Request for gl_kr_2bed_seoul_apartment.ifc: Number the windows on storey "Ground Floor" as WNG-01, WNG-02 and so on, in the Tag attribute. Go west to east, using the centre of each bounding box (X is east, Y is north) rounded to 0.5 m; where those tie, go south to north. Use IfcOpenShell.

First a look at what the model holds.

```python
import ifcopenshell
import ifcopenshell.util.element
import ifcopenshell.util.placement

model = ifcopenshell.open("gl_kr_2bed_seoul_apartment.ifc")
print(model.schema)
storey = next(s for s in model.by_type("IfcBuildingStorey") if s.Name == "Ground Floor")
windows = [e for e in ifcopenshell.util.element.get_decomposition(storey) if e.is_a("IfcWindow")]
for e in sorted(windows, key=lambda e: e.id()):
    origin = ifcopenshell.util.placement.get_local_placement(e.ObjectPlacement)[:3, 3]
    print(e.id(), e.Tag, e.Name, origin.round(2) + 0.0, sep=" | ")
```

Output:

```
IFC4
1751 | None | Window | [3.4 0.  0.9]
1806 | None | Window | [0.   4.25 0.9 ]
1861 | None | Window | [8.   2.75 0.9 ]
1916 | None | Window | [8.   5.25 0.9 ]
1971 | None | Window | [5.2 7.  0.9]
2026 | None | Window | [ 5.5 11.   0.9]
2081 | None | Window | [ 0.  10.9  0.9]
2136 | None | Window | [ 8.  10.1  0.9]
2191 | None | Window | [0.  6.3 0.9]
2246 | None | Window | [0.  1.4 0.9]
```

```python
import ifcopenshell
import ifcopenshell.geom
import ifcopenshell.util.element
import ifcopenshell.util.shape

model = ifcopenshell.open("gl_kr_2bed_seoul_apartment.ifc")
settings = ifcopenshell.geom.settings()
settings.set("use-world-coords", True)


def centre(element):
    shape = ifcopenshell.geom.create_shape(settings, element)
    return ifcopenshell.util.shape.get_bbox_centroid(shape.geometry)


storey = next(s for s in model.by_type("IfcBuildingStorey") if s.Name == "Ground Floor")
windows = [e for e in ifcopenshell.util.element.get_decomposition(storey) if e.is_a("IfcWindow")]

# Insertion points can sit at a corner or the storey origin, so sort by the geometry (in metres).
centres = {e: centre(e) for e in windows}
windows.sort(key=lambda e: (round(centres[e][0] / 0.5), centres[e][1]))

for i, e in enumerate(windows, start=1):
    number = f"WNG-{i:02d}"
    e.Tag = number
    print(e.id(), number)

model.write("gl_kr_2bed_seoul_apartment_updated.ifc")
```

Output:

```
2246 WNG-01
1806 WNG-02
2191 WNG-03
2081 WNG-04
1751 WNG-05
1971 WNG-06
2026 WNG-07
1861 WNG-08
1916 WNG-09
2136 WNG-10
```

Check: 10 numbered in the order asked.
